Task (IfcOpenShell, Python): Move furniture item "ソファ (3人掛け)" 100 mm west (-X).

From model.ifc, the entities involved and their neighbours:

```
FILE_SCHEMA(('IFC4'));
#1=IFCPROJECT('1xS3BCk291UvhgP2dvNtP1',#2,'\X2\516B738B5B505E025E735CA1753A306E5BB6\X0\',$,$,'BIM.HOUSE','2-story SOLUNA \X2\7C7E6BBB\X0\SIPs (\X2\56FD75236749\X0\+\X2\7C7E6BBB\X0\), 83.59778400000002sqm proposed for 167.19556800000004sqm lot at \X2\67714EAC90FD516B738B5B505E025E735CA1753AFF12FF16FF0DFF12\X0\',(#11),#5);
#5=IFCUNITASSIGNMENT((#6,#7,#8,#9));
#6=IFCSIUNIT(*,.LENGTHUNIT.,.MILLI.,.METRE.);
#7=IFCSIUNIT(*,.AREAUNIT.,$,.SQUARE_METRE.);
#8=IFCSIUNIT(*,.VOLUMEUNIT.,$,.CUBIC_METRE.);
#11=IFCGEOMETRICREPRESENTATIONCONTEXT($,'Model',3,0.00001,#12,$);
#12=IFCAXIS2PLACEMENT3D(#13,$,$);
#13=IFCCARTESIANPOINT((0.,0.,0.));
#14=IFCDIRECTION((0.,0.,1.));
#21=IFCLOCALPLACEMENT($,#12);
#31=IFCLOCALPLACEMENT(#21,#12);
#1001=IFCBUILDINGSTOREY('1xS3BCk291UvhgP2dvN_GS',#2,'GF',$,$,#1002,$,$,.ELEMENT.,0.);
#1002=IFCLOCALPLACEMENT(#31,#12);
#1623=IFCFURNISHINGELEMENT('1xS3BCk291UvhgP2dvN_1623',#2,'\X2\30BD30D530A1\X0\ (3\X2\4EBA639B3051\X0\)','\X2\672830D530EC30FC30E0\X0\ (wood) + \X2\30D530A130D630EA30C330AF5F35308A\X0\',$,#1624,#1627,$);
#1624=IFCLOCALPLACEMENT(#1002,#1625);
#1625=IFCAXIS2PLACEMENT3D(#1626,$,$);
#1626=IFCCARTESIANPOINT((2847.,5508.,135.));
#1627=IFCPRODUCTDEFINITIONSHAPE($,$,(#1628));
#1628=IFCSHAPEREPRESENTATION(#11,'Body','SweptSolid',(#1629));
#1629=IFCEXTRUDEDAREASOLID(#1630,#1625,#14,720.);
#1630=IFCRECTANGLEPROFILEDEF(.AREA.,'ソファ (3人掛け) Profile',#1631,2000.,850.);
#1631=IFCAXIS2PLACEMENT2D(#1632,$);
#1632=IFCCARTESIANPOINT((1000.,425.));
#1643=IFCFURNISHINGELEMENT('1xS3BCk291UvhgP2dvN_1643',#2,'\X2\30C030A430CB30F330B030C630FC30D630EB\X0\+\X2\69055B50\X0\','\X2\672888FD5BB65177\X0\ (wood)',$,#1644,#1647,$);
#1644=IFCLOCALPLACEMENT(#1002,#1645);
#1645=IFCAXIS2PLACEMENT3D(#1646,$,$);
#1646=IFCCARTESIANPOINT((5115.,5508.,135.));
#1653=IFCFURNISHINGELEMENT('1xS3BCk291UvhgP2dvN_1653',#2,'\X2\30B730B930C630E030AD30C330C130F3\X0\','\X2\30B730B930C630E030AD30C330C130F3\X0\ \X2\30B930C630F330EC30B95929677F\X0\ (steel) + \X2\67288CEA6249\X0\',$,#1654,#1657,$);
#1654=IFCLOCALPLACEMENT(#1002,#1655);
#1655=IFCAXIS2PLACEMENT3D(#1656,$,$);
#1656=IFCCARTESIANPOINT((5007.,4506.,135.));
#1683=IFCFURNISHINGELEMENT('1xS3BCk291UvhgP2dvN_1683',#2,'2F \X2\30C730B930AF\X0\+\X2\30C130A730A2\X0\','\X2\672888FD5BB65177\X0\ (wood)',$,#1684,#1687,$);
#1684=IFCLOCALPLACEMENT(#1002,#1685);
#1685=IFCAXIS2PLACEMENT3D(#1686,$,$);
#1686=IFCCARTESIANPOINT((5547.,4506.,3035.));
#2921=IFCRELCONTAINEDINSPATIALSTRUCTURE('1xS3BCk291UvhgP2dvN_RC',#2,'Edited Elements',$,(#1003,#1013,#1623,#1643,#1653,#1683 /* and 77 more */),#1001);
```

```python
import ifcopenshell
import ifcopenshell.api.geometry
import ifcopenshell.util.placement

model = ifcopenshell.open("model.ifc")

item = model.by_id(1623)
matrix = ifcopenshell.util.placement.get_local_placement(item.ObjectPlacement)
matrix[0, 3] -= 100.0
ifcopenshell.api.geometry.edit_object_placement(model, product=item, matrix=matrix, is_si=False)

print(ifcopenshell.util.placement.get_local_placement(item.ObjectPlacement).round(3) + 0.0)

model.write("model_rev.ifc")
```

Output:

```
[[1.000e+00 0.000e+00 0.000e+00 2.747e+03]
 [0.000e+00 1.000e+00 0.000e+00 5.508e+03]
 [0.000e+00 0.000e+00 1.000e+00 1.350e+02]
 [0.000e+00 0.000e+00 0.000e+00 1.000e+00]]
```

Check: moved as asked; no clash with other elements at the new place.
